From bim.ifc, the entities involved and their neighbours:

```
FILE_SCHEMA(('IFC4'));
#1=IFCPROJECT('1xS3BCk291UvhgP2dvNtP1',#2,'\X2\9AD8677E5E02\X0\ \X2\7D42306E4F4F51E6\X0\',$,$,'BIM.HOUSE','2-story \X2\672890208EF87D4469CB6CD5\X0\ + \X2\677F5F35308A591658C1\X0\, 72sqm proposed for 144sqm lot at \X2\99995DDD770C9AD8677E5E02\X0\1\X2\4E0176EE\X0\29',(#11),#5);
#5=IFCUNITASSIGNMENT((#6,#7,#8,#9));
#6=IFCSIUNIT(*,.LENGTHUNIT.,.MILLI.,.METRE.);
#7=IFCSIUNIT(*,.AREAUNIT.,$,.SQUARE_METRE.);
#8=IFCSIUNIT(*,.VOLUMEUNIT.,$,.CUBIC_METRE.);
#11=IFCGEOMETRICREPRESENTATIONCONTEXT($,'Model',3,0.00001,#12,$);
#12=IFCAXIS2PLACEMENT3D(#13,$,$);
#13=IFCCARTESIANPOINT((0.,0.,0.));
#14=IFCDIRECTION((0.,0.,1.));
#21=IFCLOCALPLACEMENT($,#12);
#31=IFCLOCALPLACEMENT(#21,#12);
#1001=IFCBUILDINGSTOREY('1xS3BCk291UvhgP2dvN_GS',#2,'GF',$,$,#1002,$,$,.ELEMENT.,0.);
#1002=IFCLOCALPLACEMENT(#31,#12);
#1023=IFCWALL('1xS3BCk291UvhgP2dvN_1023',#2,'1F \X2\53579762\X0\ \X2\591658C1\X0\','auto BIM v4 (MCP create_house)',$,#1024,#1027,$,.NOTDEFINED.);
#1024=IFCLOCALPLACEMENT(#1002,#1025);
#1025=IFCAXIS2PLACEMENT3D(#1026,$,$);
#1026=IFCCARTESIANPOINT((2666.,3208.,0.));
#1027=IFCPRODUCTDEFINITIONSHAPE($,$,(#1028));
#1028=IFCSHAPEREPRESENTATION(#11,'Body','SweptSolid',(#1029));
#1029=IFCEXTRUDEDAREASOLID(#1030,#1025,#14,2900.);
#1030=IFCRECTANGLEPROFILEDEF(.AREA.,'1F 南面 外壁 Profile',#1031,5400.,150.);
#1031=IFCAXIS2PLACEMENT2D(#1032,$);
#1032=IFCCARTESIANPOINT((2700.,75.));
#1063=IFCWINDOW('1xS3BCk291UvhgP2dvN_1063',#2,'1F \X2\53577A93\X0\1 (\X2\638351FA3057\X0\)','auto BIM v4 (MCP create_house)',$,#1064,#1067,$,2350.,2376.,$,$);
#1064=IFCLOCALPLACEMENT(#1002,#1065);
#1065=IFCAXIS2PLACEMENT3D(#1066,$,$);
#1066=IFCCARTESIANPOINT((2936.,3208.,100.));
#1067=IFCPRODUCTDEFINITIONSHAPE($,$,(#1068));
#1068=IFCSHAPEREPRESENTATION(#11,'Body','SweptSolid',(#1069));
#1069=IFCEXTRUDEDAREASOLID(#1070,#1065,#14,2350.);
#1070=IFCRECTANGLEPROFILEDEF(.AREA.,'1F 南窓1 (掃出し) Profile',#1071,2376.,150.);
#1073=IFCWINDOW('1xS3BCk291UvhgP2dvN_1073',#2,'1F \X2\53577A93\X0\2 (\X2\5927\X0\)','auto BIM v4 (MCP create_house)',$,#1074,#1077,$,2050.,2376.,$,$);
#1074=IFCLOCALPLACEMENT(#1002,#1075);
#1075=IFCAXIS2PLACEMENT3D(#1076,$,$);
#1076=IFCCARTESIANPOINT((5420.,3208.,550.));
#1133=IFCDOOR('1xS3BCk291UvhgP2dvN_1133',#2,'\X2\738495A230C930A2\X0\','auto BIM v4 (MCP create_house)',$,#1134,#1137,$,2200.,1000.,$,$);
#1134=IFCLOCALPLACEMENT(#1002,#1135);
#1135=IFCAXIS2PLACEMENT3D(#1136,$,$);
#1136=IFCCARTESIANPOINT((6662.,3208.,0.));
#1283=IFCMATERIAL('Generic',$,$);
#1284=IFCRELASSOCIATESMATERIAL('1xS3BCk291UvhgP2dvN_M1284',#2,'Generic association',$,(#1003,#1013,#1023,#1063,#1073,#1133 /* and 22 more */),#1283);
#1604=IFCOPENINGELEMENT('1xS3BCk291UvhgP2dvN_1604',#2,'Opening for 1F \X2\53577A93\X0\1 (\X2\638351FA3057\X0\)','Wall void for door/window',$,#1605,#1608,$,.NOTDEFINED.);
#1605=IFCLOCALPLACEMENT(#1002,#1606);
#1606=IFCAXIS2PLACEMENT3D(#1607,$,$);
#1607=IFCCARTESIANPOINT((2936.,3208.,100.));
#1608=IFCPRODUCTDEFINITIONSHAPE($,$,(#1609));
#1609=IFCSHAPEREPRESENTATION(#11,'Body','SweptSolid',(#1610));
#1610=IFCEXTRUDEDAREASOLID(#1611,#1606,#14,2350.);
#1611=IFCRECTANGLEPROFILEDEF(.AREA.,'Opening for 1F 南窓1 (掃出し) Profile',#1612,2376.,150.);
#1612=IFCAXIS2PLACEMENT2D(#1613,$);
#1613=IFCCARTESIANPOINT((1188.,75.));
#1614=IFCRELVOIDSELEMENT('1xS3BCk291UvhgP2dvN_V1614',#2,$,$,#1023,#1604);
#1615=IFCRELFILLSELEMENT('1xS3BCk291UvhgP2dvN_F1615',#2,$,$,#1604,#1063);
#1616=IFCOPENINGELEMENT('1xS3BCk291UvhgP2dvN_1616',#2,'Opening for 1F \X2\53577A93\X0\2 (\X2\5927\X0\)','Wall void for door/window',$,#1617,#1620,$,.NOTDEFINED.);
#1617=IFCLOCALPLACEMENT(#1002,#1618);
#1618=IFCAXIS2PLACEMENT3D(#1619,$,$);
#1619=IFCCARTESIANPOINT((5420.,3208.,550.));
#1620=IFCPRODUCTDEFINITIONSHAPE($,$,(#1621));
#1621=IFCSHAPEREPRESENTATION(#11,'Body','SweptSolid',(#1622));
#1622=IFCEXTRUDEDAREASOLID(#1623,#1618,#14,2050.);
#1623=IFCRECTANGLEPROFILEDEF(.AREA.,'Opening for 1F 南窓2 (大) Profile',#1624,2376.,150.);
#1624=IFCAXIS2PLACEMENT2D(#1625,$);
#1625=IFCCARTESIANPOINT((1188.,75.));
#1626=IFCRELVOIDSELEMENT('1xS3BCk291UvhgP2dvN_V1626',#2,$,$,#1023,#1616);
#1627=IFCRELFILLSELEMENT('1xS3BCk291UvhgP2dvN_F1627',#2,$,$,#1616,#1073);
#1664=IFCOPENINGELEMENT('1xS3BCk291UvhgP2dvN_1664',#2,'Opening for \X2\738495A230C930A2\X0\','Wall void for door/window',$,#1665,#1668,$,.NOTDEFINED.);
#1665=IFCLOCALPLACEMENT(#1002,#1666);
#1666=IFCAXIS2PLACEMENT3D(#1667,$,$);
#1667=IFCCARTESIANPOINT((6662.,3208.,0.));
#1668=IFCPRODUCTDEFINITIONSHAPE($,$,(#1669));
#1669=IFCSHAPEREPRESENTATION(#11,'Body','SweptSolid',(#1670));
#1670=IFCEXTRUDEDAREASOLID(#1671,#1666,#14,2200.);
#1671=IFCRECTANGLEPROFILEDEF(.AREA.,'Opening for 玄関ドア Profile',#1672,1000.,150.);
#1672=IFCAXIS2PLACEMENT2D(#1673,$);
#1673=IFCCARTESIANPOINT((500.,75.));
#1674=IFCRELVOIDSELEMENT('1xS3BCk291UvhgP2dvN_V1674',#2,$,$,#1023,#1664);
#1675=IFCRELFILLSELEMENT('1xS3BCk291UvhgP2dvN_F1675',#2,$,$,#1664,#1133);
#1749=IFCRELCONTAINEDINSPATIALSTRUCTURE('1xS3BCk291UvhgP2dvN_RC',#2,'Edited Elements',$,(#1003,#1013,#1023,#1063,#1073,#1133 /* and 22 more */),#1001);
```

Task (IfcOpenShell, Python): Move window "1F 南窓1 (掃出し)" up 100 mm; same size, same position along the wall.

```python
import numpy as np
import ifcopenshell
import ifcopenshell.api.geometry
import ifcopenshell.util.placement
import ifcopenshell.util.unit

model = ifcopenshell.open("bim.ifc")
unit_scale = ifcopenshell.util.unit.calculate_unit_scale(model)

window = model.by_guid("1xS3BCk291UvhgP2dvN_1063")
opening = window.FillsVoids[0].RelatingOpeningElement
dz = 0.1 / unit_scale

shift = np.array([0.0, 0.0, dz])
# The window is not placed relative to its opening, so move both.
for product in (opening, window):
    matrix = ifcopenshell.util.placement.get_local_placement(product.ObjectPlacement)
    matrix[:3, 3] += shift
    ifcopenshell.api.geometry.edit_object_placement(model, product=product, matrix=matrix, is_si=False)

print(f"moved by {dz * unit_scale:+.3f} m")

model.write("bim_v2.ifc")
```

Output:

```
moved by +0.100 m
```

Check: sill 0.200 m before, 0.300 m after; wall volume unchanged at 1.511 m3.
